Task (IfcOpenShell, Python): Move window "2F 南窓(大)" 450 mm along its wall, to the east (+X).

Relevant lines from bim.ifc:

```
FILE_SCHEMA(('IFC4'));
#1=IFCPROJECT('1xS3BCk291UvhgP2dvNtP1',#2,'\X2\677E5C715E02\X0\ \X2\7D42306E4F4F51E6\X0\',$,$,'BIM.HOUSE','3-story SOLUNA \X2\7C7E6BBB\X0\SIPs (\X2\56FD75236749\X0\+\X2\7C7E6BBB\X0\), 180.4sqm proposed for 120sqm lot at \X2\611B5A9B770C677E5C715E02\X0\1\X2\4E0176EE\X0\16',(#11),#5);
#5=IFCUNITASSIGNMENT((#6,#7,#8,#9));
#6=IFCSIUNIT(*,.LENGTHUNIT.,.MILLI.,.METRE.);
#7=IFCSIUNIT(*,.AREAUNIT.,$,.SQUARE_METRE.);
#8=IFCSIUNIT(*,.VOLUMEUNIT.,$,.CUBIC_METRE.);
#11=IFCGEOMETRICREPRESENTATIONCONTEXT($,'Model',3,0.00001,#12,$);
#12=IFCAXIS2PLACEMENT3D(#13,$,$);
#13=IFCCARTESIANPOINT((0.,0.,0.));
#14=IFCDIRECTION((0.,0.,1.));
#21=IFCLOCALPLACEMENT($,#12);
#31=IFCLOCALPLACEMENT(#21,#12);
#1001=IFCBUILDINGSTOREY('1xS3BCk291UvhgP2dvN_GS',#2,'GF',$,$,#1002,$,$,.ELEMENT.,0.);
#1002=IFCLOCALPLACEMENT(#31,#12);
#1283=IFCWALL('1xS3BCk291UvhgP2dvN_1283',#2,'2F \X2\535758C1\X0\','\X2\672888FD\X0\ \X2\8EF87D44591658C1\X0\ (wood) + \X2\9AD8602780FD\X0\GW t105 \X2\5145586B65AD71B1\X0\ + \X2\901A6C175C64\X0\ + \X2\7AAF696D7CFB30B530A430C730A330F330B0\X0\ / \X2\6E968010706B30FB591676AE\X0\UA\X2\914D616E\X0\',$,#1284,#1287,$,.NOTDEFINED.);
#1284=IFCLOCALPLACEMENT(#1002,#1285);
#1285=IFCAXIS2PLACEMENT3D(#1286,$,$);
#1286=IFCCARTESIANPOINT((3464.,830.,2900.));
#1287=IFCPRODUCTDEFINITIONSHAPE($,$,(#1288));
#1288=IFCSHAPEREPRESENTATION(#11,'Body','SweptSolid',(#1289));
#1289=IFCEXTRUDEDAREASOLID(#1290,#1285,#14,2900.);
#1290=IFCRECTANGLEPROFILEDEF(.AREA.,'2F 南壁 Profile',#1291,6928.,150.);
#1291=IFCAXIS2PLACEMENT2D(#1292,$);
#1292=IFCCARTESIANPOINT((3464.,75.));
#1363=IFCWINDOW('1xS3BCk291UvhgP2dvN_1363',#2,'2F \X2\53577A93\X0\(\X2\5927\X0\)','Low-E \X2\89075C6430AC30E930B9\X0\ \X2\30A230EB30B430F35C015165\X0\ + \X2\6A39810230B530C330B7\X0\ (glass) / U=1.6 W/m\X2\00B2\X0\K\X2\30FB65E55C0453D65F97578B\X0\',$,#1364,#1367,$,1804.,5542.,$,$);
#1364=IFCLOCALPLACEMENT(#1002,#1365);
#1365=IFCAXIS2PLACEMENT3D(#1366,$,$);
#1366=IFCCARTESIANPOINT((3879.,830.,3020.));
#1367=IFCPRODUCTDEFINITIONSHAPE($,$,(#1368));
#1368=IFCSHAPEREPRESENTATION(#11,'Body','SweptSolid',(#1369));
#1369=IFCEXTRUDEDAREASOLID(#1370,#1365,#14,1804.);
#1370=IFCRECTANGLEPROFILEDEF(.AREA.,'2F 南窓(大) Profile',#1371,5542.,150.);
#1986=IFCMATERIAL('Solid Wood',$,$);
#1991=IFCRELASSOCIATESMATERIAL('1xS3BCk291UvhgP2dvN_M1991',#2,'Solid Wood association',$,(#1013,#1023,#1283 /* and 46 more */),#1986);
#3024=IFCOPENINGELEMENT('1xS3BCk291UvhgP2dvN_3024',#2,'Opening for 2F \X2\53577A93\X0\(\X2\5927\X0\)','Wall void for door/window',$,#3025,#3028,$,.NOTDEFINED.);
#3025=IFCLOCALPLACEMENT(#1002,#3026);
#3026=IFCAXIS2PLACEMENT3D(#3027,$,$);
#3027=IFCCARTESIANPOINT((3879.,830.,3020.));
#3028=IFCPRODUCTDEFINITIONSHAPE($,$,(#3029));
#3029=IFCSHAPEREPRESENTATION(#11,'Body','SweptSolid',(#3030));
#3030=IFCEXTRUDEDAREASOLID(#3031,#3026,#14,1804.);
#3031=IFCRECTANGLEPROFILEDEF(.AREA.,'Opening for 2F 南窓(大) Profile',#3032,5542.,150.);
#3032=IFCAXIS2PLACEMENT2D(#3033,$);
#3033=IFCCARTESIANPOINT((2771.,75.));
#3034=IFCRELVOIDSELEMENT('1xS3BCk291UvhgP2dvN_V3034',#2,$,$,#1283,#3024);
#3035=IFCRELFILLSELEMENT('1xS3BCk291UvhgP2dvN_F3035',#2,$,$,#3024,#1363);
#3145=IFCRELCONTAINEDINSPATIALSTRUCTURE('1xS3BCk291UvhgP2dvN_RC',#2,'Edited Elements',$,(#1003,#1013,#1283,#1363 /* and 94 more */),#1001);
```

```python
import ifcopenshell
import ifcopenshell.api.geometry
import ifcopenshell.util.placement
import ifcopenshell.util.unit

model = ifcopenshell.open("bim.ifc")
unit_scale = ifcopenshell.util.unit.calculate_unit_scale(model)

window = model.by_guid("1xS3BCk291UvhgP2dvN_1363")
opening = window.FillsVoids[0].RelatingOpeningElement
wall = opening.VoidsElements[0].RelatingBuildingElement

wall_matrix = ifcopenshell.util.placement.get_local_placement(wall.ObjectPlacement)
shift = wall_matrix[:3, 0] * 0.45 / unit_scale
before = ifcopenshell.util.placement.get_local_placement(window.ObjectPlacement)[:3, 3].copy()

# The window is not placed relative to its opening, so move both.
for product in (opening, window):
    matrix = ifcopenshell.util.placement.get_local_placement(product.ObjectPlacement)
    matrix[:3, 3] += shift
    ifcopenshell.api.geometry.edit_object_placement(model, product=product, matrix=matrix, is_si=False)

after = ifcopenshell.util.placement.get_local_placement(window.ObjectPlacement)[:3, 3]
print("window moved by", (after - before).round(3) + 0.0)

model.write("bim_rev.ifc")
```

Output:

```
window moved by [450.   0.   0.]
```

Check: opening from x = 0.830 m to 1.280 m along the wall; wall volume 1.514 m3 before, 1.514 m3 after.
